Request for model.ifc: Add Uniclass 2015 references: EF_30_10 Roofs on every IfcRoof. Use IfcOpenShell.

First a look at what the model holds.

```python
import ifcopenshell

model = ifcopenshell.open("model.ifc")
print(model.schema)
print("classifications:", [c.Name for c in model.by_type("IfcClassification")])
for ifc_class in ("IfcDoor", "IfcRoof", "IfcStair", "IfcWall", "IfcWindow"):
    print(ifc_class, len(model.by_type(ifc_class)))
```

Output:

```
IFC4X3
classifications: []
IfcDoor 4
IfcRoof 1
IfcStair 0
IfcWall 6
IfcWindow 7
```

```python
import ifcopenshell
import ifcopenshell.api.classification

model = ifcopenshell.open("model.ifc")

system = ifcopenshell.api.classification.add_classification(model, classification="Uniclass 2015")

codes = {
    "IfcRoof": ("EF_30_10", "Roofs"),
}
for ifc_class, (code, name) in codes.items():
    products = model.by_type(ifc_class)
    ifcopenshell.api.classification.add_reference(
        model, products=products, classification=system, identification=code, name=name
    )
    print(code, len(products))

model.write("model-out.ifc")
```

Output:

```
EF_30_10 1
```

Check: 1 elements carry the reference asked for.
